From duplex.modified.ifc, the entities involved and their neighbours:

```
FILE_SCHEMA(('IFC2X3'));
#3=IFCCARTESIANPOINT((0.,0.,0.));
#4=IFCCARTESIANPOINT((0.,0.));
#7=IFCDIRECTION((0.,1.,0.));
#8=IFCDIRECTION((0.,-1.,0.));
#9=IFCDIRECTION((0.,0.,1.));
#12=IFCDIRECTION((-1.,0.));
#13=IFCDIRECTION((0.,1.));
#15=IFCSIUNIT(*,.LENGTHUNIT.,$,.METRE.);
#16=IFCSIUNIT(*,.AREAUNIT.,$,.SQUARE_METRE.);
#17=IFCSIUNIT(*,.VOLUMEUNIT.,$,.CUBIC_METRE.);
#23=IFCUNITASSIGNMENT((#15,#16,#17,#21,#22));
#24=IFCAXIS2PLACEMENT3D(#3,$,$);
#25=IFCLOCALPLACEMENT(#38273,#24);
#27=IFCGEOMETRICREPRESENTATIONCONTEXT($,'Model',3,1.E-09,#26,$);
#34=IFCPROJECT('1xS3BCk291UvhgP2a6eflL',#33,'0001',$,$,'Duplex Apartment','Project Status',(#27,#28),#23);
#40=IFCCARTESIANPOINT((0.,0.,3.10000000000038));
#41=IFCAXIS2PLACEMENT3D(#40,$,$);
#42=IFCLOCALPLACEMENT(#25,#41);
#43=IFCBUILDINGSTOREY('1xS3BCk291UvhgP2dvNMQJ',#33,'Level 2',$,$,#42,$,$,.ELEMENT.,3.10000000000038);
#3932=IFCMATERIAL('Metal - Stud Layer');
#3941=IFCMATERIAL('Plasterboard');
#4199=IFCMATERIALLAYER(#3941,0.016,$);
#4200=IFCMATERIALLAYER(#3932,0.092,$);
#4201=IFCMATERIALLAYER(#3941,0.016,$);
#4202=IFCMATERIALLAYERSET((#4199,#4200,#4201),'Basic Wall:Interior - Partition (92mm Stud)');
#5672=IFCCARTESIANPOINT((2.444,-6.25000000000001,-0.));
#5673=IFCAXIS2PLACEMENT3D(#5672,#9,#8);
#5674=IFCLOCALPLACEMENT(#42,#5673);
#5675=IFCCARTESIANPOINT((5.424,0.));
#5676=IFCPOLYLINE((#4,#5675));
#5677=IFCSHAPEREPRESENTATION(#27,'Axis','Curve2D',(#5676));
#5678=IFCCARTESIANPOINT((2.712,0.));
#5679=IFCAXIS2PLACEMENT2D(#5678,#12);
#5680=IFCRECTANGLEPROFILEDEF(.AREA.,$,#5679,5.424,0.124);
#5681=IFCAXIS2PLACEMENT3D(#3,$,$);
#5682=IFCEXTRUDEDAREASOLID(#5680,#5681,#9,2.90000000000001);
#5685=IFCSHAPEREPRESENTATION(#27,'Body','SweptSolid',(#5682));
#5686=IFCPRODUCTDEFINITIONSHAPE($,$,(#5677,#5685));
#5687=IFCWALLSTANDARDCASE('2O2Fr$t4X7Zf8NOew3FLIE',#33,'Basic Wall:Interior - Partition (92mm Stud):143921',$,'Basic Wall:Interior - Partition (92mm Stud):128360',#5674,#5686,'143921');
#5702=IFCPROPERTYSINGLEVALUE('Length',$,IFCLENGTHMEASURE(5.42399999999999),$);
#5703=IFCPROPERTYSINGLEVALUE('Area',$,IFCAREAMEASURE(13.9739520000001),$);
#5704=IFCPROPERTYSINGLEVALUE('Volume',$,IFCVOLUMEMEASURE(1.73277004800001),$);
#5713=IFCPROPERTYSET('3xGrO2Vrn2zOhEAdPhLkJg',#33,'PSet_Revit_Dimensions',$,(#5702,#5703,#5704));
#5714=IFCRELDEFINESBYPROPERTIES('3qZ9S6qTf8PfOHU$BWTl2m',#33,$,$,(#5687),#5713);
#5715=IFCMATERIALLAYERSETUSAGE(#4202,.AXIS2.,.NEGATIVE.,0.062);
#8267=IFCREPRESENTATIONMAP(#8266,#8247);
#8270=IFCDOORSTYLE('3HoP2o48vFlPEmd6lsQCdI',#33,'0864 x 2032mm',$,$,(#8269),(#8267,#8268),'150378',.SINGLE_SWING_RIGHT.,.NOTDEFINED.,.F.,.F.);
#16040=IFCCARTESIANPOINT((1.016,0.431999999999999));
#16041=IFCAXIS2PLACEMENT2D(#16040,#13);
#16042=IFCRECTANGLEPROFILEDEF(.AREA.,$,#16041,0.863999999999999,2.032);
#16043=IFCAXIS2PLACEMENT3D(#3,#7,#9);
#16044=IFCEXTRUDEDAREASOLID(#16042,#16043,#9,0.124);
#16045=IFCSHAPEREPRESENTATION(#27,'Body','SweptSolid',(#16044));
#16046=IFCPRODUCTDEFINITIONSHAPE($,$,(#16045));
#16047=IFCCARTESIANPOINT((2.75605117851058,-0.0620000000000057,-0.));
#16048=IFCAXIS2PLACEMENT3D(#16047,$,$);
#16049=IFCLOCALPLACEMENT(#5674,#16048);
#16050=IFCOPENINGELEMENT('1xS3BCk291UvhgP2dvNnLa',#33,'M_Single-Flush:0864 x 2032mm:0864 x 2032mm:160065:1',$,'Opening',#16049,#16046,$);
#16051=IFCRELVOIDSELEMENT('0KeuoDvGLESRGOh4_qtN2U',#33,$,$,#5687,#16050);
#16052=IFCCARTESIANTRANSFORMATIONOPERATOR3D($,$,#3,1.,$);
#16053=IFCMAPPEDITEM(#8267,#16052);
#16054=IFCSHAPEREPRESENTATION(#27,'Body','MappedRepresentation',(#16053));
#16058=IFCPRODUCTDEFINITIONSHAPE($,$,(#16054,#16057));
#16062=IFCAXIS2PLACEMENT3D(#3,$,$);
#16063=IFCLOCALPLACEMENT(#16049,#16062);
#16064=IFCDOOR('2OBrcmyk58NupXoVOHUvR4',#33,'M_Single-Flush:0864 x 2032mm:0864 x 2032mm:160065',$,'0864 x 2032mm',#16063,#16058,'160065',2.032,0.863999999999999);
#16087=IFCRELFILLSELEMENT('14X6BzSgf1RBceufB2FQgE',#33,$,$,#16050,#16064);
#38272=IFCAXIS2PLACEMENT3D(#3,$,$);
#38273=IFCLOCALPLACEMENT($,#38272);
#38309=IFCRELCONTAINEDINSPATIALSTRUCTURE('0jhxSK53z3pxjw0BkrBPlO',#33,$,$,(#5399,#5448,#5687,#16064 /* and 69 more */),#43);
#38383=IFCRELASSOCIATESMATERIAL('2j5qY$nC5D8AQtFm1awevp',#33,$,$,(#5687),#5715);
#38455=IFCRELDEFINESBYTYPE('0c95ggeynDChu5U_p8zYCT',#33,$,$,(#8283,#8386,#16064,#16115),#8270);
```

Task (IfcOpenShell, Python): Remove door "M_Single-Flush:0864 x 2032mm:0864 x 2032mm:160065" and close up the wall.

```python
import ifcopenshell
import ifcopenshell.api.feature
import ifcopenshell.api.pset
import ifcopenshell.api.root
import ifcopenshell.geom
import ifcopenshell.util.element
import ifcopenshell.util.shape
import ifcopenshell.util.unit

model = ifcopenshell.open("duplex.modified.ifc")
area_scale = ifcopenshell.util.unit.calculate_unit_scale(model, "AREAUNIT")
volume_scale = ifcopenshell.util.unit.calculate_unit_scale(model, "VOLUMEUNIT")
settings = ifcopenshell.geom.settings()


def volume(element):
    """Net volume in cubic metres, openings subtracted."""
    shape = ifcopenshell.geom.create_shape(settings, element)
    return ifcopenshell.util.shape.get_volume(shape.geometry)


door = model.by_guid("2OBrcmyk58NupXoVOHUvR4")
opening = door.FillsVoids[0].RelatingOpeningElement
wall = opening.VoidsElements[0].RelatingBuildingElement
before = volume(wall)

ifcopenshell.api.root.remove_product(model, product=door)
ifcopenshell.api.feature.remove_feature(model, feature=opening)

after = volume(wall)
thickness = 0.124  # wall thickness in metres

# Update the wall's stored quantities.
pset = model.by_id(ifcopenshell.util.element.get_pset(wall, "PSet_Revit_Dimensions", should_inherit=False)["id"])
ifcopenshell.api.pset.edit_pset(model, pset=pset, properties={
    "Area": model.create_entity("IfcAreaMeasure", after / thickness / area_scale),
    "Volume": model.create_entity("IfcVolumeMeasure", after / volume_scale),
})

print(f"wall volume {before:.3f} -> {after:.3f} m3")

model.write("duplex.modified_v2.ifc")
```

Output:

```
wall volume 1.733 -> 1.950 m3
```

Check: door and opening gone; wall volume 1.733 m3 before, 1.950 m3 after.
